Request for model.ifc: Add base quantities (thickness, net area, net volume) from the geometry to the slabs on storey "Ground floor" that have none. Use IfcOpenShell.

First a look at what the model holds.

```python
import ifcopenshell
import ifcopenshell.util.element
import ifcopenshell.util.unit

model = ifcopenshell.open("model.ifc")
print(model.schema)
for unit_type in ("LENGTHUNIT", "AREAUNIT", "VOLUMEUNIT"):
    print(unit_type, ifcopenshell.util.unit.calculate_unit_scale(model, unit_type))
storey = next(s for s in model.by_type("IfcBuildingStorey") if s.Name == "Ground floor")
slabs = [e for e in ifcopenshell.util.element.get_decomposition(storey) if e.is_a("IfcSlab")]
for e in sorted(slabs, key=lambda e: e.id()):
    print(e.id(), e.is_a(), e.Name, list(ifcopenshell.util.element.get_psets(e, qtos_only=True)), sep=" | ")
```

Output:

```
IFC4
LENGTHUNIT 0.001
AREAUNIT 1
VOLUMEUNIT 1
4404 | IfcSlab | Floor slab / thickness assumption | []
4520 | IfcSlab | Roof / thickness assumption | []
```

```python
import ifcopenshell
import ifcopenshell.api.pset
import ifcopenshell.geom
import ifcopenshell.util.element
import ifcopenshell.util.shape
import ifcopenshell.util.unit

model = ifcopenshell.open("model.ifc")
unit_scale = ifcopenshell.util.unit.calculate_unit_scale(model)
area_scale = ifcopenshell.util.unit.calculate_unit_scale(model, "AREAUNIT")
volume_scale = ifcopenshell.util.unit.calculate_unit_scale(model, "VOLUMEUNIT")
settings = ifcopenshell.geom.settings()

storey = next(s for s in model.by_type("IfcBuildingStorey") if s.Name == "Ground floor")
slabs = [e for e in ifcopenshell.util.element.get_decomposition(storey) if e.is_a("IfcSlab")]

for e in sorted(slabs, key=lambda e: e.id()):
    if ifcopenshell.util.element.get_psets(e, qtos_only=True, should_inherit=False):
        continue
    # Geometry comes back in metres, in the element's own axes.
    shape = ifcopenshell.geom.create_shape(settings, e)
    values = {
        "Width": ifcopenshell.util.shape.get_z(shape.geometry) / unit_scale,
        "NetArea": ifcopenshell.util.shape.get_footprint_area(shape.geometry) / area_scale,
        "NetVolume": ifcopenshell.util.shape.get_volume(shape.geometry) / volume_scale,
    }
    qto = ifcopenshell.api.pset.add_qto(model, product=e, name="Qto_SlabBaseQuantities")
    ifcopenshell.api.pset.edit_qto(model, qto=qto, properties=values)
    print(e.id(), {k: round(v, 3) for k, v in values.items()})

model.write("model_v2.ifc")
```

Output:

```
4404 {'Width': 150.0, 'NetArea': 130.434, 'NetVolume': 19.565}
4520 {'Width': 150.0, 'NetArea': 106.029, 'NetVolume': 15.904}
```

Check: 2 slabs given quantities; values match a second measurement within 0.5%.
